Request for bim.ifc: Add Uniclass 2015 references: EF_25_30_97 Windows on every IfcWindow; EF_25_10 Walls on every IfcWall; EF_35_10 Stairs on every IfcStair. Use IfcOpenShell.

First a look at what the model holds.

```python
import ifcopenshell

model = ifcopenshell.open("bim.ifc")
print(model.schema)
print("classifications:", [c.Name for c in model.by_type("IfcClassification")])
for ifc_class in ("IfcDoor", "IfcRoof", "IfcStair", "IfcWall", "IfcWindow"):
    print(ifc_class, len(model.by_type(ifc_class)))
```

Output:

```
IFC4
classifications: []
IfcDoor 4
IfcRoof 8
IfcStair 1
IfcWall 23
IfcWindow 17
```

```python
import ifcopenshell
import ifcopenshell.api.classification

model = ifcopenshell.open("bim.ifc")

system = ifcopenshell.api.classification.add_classification(model, classification="Uniclass 2015")

codes = {
    "IfcWindow": ("EF_25_30_97", "Windows"),
    "IfcWall": ("EF_25_10", "Walls"),
    "IfcStair": ("EF_35_10", "Stairs"),
}
for ifc_class, (code, name) in codes.items():
    products = model.by_type(ifc_class)
    ifcopenshell.api.classification.add_reference(
        model, products=products, classification=system, identification=code, name=name
    )
    print(code, len(products))

model.write("bim_updated.ifc")
```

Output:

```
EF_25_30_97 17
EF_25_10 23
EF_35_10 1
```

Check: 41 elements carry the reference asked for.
